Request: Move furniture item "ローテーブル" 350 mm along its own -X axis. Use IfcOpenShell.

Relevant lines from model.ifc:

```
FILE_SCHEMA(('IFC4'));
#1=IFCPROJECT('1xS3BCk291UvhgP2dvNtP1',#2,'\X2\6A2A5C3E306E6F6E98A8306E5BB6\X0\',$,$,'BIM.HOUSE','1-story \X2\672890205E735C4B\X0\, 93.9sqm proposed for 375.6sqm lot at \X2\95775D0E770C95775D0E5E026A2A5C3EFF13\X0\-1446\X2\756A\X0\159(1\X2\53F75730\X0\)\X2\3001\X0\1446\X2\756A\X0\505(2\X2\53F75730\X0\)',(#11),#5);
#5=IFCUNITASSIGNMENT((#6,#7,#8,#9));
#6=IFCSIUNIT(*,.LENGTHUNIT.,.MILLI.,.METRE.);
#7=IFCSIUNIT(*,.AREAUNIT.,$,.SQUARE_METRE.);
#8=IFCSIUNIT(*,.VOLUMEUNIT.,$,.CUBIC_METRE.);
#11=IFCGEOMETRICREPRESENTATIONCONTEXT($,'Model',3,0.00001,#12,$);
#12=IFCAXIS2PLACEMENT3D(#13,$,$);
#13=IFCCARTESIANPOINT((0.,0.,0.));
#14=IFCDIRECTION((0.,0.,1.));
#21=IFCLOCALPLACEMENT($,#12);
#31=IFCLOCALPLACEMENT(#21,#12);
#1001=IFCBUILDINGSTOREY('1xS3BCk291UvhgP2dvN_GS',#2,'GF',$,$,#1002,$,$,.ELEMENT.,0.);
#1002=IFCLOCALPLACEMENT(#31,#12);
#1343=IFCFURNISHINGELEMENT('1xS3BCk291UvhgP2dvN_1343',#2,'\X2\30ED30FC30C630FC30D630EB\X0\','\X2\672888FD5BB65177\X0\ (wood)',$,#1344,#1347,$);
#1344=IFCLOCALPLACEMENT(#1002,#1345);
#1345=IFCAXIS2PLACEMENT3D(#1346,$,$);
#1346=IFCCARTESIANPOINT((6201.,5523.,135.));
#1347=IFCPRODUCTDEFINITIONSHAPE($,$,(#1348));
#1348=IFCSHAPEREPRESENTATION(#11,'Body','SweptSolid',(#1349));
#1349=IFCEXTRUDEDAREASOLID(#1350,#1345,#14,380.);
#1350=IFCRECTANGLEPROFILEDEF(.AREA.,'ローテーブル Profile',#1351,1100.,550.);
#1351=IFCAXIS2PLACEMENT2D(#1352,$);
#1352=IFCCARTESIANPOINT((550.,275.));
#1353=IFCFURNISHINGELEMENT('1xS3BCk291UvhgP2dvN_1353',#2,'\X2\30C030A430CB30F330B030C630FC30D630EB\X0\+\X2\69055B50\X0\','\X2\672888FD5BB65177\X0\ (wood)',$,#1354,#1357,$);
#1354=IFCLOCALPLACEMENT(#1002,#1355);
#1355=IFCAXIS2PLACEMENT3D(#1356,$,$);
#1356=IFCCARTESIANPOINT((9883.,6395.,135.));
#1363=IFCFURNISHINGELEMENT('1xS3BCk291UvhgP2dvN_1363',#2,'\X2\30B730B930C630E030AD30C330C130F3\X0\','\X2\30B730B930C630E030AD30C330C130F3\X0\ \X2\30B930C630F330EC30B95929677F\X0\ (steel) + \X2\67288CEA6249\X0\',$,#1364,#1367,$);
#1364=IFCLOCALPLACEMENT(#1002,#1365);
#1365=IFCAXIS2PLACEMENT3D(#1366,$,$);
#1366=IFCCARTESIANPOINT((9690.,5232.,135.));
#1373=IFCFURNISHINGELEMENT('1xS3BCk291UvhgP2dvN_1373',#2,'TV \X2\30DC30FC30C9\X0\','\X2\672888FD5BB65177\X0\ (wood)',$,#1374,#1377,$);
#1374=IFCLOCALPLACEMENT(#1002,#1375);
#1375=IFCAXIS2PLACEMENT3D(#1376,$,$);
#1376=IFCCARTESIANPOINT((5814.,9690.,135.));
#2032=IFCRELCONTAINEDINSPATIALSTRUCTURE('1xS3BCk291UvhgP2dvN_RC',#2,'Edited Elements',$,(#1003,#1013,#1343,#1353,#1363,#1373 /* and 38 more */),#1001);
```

```python
import ifcopenshell
import ifcopenshell.api.geometry
import ifcopenshell.util.placement
import ifcopenshell.util.unit

model = ifcopenshell.open("model.ifc")
unit_scale = ifcopenshell.util.unit.calculate_unit_scale(model)

item = model.by_id(1343)
matrix = ifcopenshell.util.placement.get_local_placement(item.ObjectPlacement)
matrix[:3, 3] -= matrix[:3, 0] * 0.35 / unit_scale
ifcopenshell.api.geometry.edit_object_placement(model, product=item, matrix=matrix, is_si=False)

print(ifcopenshell.util.placement.get_local_placement(item.ObjectPlacement).round(3) + 0.0)

model.write("model_updated.ifc")
```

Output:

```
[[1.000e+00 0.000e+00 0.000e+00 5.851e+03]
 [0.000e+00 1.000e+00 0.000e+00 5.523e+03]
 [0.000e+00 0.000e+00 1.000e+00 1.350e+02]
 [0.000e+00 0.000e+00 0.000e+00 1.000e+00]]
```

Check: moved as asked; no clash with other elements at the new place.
